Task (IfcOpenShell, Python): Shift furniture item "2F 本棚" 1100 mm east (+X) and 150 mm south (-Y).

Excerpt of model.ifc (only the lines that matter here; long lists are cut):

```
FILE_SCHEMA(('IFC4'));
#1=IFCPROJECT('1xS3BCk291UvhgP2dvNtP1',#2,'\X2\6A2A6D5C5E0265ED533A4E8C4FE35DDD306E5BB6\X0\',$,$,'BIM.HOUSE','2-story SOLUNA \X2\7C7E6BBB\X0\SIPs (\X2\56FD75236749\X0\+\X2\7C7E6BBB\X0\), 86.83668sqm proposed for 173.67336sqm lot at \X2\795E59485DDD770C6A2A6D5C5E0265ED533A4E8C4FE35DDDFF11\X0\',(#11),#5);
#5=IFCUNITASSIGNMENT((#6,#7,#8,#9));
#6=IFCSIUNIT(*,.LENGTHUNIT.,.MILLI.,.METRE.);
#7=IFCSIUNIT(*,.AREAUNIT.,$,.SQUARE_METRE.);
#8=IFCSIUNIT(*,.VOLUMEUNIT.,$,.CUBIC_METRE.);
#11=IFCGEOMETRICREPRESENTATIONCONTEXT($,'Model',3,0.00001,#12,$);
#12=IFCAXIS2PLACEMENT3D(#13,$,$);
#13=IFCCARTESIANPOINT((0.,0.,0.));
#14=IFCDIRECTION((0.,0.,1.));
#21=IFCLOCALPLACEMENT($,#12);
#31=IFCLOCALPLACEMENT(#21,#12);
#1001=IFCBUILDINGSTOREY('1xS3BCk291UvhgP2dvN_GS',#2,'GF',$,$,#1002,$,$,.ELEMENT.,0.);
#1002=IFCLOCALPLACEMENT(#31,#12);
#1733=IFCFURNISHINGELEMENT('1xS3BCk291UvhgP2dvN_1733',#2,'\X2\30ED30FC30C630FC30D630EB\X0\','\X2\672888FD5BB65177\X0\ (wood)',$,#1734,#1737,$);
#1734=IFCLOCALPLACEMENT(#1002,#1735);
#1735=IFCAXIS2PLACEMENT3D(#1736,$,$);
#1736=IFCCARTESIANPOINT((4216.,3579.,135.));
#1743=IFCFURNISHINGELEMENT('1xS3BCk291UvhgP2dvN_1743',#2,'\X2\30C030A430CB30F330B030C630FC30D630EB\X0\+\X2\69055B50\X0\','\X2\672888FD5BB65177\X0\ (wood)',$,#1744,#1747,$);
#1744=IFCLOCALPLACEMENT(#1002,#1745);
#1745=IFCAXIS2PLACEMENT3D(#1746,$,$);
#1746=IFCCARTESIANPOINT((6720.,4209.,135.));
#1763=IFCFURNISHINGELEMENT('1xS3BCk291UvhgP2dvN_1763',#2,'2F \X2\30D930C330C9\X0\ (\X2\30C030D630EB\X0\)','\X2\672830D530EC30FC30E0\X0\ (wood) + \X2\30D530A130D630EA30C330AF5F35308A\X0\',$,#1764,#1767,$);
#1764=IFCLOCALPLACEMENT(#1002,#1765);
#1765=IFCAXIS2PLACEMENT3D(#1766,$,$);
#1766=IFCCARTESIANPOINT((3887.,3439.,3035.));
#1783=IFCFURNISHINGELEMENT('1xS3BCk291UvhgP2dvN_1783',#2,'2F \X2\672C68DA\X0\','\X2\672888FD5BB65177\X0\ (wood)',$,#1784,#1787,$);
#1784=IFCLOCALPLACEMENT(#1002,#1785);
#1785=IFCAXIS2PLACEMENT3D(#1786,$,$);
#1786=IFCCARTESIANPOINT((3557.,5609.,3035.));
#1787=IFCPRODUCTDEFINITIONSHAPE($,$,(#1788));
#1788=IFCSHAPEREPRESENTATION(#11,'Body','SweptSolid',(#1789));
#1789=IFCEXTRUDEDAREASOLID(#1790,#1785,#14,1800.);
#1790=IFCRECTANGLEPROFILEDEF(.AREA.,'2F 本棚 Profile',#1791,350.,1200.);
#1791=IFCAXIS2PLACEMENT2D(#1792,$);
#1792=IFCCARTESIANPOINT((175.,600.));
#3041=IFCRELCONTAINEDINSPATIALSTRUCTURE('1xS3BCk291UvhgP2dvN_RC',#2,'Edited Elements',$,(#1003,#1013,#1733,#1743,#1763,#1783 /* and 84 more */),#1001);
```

```python
import ifcopenshell
import ifcopenshell.api.geometry
import ifcopenshell.util.placement

model = ifcopenshell.open("model.ifc")

item = model.by_guid("1xS3BCk291UvhgP2dvN_1783")
matrix = ifcopenshell.util.placement.get_local_placement(item.ObjectPlacement)
matrix[0, 3] += 1100.0
matrix[1, 3] -= 150.0
ifcopenshell.api.geometry.edit_object_placement(model, product=item, matrix=matrix, is_si=False)

print(ifcopenshell.util.placement.get_local_placement(item.ObjectPlacement).round(3) + 0.0)

model.write("model_updated.ifc")
```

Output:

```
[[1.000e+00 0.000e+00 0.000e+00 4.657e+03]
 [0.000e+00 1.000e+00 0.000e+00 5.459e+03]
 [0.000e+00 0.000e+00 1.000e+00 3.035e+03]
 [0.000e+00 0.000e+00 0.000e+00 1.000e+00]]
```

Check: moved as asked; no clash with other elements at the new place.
